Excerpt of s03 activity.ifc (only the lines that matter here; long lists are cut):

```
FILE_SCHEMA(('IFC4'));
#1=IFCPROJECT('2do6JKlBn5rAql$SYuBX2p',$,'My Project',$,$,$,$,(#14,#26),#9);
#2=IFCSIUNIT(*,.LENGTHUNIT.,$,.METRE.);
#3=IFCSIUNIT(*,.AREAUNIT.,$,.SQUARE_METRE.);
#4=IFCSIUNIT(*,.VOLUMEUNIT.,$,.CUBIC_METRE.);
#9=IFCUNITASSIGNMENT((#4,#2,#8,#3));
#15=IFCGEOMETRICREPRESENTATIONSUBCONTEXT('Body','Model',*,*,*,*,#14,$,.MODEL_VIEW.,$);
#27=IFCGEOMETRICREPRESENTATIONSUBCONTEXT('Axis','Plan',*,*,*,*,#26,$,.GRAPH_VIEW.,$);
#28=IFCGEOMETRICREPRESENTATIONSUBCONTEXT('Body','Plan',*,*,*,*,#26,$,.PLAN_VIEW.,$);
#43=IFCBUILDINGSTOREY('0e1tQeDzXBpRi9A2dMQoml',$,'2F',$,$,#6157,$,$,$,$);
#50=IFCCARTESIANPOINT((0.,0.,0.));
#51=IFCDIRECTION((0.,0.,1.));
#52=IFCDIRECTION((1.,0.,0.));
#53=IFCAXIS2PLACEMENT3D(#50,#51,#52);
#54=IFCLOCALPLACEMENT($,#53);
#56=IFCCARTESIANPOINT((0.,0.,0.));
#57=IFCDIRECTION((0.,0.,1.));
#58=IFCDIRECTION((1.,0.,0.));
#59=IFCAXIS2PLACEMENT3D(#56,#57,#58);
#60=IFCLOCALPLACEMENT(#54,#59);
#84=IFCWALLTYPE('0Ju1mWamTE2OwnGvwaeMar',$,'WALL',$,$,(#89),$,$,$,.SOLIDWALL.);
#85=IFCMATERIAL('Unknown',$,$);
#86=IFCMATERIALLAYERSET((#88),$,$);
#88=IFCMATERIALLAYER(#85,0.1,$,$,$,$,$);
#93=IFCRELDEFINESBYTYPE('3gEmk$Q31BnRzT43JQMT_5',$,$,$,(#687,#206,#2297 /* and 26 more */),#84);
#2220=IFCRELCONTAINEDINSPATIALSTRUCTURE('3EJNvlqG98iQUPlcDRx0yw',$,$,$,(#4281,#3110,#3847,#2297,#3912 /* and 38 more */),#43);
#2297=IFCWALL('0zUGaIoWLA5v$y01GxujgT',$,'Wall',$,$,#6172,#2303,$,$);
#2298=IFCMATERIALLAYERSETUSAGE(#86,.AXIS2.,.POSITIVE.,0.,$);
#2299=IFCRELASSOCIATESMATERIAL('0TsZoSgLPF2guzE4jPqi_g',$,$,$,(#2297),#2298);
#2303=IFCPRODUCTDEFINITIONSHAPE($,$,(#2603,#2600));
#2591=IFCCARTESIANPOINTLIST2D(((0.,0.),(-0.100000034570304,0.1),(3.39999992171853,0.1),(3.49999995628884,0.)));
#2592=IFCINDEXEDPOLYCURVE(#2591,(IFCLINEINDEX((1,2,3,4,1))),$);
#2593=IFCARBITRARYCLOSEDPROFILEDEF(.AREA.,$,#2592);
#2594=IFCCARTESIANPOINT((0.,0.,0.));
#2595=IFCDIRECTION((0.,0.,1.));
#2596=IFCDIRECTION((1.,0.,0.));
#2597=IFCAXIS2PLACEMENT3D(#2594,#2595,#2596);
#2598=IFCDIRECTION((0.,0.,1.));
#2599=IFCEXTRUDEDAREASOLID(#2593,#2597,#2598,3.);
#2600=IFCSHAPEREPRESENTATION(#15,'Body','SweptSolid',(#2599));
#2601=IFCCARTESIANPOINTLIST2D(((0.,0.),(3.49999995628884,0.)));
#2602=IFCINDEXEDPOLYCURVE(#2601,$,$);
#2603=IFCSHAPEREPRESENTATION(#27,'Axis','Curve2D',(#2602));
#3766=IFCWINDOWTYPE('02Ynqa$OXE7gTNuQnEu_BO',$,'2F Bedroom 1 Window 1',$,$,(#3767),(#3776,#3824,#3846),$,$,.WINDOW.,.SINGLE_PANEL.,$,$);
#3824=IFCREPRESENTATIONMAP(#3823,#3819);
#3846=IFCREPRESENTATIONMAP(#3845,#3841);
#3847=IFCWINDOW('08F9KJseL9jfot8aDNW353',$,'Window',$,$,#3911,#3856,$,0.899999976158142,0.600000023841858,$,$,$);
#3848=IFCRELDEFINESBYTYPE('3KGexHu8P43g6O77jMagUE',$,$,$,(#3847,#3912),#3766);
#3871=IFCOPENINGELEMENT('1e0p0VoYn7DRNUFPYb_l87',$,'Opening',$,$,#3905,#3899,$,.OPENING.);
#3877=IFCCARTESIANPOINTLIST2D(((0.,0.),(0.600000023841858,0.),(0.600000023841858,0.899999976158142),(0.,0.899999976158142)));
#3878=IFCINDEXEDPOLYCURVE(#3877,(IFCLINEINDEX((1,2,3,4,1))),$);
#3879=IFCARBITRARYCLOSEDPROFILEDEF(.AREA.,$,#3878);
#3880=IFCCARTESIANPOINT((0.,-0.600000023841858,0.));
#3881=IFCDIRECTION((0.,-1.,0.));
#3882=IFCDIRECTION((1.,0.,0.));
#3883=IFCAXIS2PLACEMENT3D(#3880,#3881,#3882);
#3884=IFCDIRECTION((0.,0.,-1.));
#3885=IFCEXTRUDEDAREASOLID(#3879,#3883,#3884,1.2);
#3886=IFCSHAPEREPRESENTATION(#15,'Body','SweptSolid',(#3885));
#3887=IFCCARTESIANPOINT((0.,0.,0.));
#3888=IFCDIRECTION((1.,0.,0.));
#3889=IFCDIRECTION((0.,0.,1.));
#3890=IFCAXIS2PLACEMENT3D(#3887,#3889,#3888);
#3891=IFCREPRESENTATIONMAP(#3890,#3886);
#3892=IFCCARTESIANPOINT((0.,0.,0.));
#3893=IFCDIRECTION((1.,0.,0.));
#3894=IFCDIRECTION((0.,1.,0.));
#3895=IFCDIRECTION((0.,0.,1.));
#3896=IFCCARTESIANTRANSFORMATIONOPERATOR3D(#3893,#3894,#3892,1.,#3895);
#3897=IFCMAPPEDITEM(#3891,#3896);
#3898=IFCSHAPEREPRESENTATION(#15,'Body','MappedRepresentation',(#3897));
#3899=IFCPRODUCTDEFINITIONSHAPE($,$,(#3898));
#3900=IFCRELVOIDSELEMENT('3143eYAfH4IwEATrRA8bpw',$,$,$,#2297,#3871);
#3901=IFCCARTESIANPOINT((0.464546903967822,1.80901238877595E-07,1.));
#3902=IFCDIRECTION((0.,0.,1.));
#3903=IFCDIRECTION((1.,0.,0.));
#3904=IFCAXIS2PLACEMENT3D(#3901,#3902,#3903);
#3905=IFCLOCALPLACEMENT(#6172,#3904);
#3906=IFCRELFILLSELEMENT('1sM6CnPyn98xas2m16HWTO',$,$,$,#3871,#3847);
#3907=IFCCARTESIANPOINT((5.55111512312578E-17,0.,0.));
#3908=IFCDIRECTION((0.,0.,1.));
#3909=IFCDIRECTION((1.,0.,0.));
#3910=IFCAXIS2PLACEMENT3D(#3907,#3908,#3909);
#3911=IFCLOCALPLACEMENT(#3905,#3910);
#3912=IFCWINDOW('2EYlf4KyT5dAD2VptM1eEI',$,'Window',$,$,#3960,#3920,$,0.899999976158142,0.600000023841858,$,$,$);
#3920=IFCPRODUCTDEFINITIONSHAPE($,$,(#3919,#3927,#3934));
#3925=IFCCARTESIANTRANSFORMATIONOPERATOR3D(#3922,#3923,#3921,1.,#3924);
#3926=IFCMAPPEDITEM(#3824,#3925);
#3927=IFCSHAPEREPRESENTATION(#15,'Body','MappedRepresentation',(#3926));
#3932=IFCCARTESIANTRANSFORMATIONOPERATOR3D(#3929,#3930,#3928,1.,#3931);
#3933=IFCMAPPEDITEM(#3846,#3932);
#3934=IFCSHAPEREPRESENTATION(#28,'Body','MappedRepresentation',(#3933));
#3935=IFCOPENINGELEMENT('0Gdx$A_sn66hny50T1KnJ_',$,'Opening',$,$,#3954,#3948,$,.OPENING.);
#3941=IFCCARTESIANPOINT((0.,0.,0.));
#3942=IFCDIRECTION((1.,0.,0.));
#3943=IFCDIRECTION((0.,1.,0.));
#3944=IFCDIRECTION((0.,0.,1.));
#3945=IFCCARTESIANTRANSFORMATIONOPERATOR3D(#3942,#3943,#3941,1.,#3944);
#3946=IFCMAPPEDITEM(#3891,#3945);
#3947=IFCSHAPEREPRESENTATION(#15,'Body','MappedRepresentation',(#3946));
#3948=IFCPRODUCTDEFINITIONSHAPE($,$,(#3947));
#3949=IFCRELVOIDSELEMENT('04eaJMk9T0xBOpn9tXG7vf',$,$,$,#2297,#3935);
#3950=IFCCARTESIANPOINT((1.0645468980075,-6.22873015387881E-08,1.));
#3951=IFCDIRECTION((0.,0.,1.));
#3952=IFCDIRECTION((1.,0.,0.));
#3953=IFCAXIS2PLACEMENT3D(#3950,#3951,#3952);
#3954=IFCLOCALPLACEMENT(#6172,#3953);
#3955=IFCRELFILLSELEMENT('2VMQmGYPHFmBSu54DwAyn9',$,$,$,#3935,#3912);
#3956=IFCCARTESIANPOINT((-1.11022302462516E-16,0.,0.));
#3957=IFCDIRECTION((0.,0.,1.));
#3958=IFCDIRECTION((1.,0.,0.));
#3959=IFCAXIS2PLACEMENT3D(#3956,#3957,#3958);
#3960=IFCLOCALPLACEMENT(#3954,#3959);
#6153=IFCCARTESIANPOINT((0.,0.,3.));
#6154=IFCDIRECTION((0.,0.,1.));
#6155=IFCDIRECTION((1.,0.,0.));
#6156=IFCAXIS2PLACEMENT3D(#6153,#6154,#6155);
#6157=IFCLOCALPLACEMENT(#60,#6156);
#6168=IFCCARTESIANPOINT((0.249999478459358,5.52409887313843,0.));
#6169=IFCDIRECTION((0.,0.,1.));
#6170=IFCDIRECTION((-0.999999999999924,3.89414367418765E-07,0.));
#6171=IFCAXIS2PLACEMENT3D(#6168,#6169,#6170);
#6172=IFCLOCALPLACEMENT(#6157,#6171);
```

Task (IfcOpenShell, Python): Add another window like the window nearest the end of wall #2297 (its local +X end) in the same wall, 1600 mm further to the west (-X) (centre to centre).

```python
import ifcopenshell
import ifcopenshell.api.feature
import ifcopenshell.api.geometry
import ifcopenshell.api.root
import ifcopenshell.geom
import ifcopenshell.util.element
import ifcopenshell.util.placement
import ifcopenshell.util.shape
import ifcopenshell.util.unit

model = ifcopenshell.open("s03 activity.ifc")
unit_scale = ifcopenshell.util.unit.calculate_unit_scale(model)
settings = ifcopenshell.geom.settings()


def volume(element):
    """Net volume in cubic metres, openings subtracted."""
    shape = ifcopenshell.geom.create_shape(settings, element)
    return ifcopenshell.util.shape.get_volume(shape.geometry)


window = model.by_guid("2EYlf4KyT5dAD2VptM1eEI")
opening = window.FillsVoids[0].RelatingOpeningElement
wall = opening.VoidsElements[0].RelatingBuildingElement
before = volume(wall)
shift = ifcopenshell.util.placement.get_local_placement(wall.ObjectPlacement)[:3, 0] * 1.6 / unit_scale

# copy_class copies the void relationship, type, container and properties, but no geometry.
new_opening = ifcopenshell.api.root.copy_class(model, product=opening)
new_opening.Representation = ifcopenshell.util.element.copy_deep(
    model, opening.Representation, exclude=["IfcGeometricRepresentationContext", "IfcRepresentationMap"]
)
new_window = ifcopenshell.api.root.copy_class(model, product=window)
new_window.Representation = ifcopenshell.util.element.copy_deep(
    model, window.Representation, exclude=["IfcGeometricRepresentationContext", "IfcRepresentationMap"]
)
ifcopenshell.api.feature.add_filling(model, opening=new_opening, element=new_window)

for old, new in ((opening, new_opening), (window, new_window)):
    matrix = ifcopenshell.util.placement.get_local_placement(old.ObjectPlacement)
    matrix[:3, 3] += shift
    ifcopenshell.api.geometry.edit_object_placement(model, product=new, matrix=matrix, is_si=False)

after = volume(wall)

print(f"wall volume {before:.3f} -> {after:.3f} m3")

model.write("s03 activity-out.ifc")
```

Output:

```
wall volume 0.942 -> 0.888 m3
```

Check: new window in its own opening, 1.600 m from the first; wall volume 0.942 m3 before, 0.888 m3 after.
